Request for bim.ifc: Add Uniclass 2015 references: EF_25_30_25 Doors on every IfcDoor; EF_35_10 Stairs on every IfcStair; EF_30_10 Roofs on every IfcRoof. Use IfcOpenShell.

First a look at what the model holds.

```python
import ifcopenshell

model = ifcopenshell.open("bim.ifc")
print(model.schema)
print("classifications:", [c.Name for c in model.by_type("IfcClassification")])
for ifc_class in ("IfcDoor", "IfcRoof", "IfcStair", "IfcWall", "IfcWindow"):
    print(ifc_class, len(model.by_type(ifc_class)))
```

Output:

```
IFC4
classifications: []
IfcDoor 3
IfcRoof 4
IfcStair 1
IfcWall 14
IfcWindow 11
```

```python
import ifcopenshell
import ifcopenshell.api.classification

model = ifcopenshell.open("bim.ifc")

system = ifcopenshell.api.classification.add_classification(model, classification="Uniclass 2015")

codes = {
    "IfcDoor": ("EF_25_30_25", "Doors"),
    "IfcStair": ("EF_35_10", "Stairs"),
    "IfcRoof": ("EF_30_10", "Roofs"),
}
for ifc_class, (code, name) in codes.items():
    products = model.by_type(ifc_class)
    ifcopenshell.api.classification.add_reference(
        model, products=products, classification=system, identification=code, name=name
    )
    print(code, len(products))

model.write("bim_v2.ifc")
```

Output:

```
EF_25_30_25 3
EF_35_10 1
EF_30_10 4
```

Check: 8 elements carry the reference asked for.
